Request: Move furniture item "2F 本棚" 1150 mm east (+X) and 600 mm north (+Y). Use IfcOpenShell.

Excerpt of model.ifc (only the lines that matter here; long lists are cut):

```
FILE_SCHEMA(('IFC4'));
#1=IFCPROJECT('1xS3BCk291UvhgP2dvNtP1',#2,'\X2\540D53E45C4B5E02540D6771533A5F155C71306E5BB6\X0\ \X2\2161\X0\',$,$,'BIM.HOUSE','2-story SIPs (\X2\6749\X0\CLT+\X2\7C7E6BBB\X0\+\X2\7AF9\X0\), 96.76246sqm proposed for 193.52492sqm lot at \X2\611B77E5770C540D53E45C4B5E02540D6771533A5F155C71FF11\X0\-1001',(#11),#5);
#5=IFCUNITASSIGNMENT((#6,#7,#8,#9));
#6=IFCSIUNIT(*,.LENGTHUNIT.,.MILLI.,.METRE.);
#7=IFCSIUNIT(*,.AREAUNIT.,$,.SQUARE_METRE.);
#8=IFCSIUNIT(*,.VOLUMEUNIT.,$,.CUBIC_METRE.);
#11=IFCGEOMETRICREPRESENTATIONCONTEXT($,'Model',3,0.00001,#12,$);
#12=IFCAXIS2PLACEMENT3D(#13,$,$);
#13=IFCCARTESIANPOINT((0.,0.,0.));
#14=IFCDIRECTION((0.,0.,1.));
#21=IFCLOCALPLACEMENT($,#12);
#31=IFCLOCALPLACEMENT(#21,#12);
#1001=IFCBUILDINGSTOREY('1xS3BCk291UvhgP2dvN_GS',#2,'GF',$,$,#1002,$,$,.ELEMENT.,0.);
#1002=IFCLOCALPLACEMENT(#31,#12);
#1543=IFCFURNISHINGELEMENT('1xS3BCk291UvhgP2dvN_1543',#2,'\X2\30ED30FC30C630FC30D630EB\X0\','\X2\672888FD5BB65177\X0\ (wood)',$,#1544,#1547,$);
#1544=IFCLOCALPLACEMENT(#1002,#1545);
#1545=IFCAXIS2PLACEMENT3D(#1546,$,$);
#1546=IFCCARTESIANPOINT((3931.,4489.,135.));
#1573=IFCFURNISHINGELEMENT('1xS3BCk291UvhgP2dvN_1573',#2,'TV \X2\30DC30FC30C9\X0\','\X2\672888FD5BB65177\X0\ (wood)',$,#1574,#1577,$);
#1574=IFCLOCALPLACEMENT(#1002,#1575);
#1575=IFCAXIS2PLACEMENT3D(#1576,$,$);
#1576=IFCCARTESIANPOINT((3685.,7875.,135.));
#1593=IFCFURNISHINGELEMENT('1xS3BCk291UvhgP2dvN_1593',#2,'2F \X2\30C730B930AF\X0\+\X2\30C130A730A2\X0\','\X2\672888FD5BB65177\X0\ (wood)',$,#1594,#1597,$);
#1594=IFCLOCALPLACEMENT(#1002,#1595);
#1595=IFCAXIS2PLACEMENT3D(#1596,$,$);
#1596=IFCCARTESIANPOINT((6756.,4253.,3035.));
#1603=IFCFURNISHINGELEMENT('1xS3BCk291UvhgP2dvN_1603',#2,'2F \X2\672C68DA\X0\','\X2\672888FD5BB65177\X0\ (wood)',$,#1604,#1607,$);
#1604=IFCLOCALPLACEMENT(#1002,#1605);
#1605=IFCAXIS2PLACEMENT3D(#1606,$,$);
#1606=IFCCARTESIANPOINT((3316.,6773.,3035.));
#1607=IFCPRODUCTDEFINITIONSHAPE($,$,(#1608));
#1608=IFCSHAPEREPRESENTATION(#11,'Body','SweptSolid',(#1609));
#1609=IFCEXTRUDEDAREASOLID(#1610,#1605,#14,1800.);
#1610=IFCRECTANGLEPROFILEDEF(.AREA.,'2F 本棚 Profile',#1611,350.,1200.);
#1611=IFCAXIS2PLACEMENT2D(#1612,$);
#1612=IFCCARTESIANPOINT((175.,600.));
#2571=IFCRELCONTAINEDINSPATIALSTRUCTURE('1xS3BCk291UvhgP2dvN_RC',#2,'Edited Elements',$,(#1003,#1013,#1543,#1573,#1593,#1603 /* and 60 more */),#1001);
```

```python
import ifcopenshell
import ifcopenshell.api.geometry
import ifcopenshell.util.placement

model = ifcopenshell.open("model.ifc")

item = model.by_guid("1xS3BCk291UvhgP2dvN_1603")
matrix = ifcopenshell.util.placement.get_local_placement(item.ObjectPlacement)
matrix[0, 3] += 1150.0
matrix[1, 3] += 600.0
ifcopenshell.api.geometry.edit_object_placement(model, product=item, matrix=matrix, is_si=False)

print(ifcopenshell.util.placement.get_local_placement(item.ObjectPlacement).round(3) + 0.0)

model.write("model_rev.ifc")
```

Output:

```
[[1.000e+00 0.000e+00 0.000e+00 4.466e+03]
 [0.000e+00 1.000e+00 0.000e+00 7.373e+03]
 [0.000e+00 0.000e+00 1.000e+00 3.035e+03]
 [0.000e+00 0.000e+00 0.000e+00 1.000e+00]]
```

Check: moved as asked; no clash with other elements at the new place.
